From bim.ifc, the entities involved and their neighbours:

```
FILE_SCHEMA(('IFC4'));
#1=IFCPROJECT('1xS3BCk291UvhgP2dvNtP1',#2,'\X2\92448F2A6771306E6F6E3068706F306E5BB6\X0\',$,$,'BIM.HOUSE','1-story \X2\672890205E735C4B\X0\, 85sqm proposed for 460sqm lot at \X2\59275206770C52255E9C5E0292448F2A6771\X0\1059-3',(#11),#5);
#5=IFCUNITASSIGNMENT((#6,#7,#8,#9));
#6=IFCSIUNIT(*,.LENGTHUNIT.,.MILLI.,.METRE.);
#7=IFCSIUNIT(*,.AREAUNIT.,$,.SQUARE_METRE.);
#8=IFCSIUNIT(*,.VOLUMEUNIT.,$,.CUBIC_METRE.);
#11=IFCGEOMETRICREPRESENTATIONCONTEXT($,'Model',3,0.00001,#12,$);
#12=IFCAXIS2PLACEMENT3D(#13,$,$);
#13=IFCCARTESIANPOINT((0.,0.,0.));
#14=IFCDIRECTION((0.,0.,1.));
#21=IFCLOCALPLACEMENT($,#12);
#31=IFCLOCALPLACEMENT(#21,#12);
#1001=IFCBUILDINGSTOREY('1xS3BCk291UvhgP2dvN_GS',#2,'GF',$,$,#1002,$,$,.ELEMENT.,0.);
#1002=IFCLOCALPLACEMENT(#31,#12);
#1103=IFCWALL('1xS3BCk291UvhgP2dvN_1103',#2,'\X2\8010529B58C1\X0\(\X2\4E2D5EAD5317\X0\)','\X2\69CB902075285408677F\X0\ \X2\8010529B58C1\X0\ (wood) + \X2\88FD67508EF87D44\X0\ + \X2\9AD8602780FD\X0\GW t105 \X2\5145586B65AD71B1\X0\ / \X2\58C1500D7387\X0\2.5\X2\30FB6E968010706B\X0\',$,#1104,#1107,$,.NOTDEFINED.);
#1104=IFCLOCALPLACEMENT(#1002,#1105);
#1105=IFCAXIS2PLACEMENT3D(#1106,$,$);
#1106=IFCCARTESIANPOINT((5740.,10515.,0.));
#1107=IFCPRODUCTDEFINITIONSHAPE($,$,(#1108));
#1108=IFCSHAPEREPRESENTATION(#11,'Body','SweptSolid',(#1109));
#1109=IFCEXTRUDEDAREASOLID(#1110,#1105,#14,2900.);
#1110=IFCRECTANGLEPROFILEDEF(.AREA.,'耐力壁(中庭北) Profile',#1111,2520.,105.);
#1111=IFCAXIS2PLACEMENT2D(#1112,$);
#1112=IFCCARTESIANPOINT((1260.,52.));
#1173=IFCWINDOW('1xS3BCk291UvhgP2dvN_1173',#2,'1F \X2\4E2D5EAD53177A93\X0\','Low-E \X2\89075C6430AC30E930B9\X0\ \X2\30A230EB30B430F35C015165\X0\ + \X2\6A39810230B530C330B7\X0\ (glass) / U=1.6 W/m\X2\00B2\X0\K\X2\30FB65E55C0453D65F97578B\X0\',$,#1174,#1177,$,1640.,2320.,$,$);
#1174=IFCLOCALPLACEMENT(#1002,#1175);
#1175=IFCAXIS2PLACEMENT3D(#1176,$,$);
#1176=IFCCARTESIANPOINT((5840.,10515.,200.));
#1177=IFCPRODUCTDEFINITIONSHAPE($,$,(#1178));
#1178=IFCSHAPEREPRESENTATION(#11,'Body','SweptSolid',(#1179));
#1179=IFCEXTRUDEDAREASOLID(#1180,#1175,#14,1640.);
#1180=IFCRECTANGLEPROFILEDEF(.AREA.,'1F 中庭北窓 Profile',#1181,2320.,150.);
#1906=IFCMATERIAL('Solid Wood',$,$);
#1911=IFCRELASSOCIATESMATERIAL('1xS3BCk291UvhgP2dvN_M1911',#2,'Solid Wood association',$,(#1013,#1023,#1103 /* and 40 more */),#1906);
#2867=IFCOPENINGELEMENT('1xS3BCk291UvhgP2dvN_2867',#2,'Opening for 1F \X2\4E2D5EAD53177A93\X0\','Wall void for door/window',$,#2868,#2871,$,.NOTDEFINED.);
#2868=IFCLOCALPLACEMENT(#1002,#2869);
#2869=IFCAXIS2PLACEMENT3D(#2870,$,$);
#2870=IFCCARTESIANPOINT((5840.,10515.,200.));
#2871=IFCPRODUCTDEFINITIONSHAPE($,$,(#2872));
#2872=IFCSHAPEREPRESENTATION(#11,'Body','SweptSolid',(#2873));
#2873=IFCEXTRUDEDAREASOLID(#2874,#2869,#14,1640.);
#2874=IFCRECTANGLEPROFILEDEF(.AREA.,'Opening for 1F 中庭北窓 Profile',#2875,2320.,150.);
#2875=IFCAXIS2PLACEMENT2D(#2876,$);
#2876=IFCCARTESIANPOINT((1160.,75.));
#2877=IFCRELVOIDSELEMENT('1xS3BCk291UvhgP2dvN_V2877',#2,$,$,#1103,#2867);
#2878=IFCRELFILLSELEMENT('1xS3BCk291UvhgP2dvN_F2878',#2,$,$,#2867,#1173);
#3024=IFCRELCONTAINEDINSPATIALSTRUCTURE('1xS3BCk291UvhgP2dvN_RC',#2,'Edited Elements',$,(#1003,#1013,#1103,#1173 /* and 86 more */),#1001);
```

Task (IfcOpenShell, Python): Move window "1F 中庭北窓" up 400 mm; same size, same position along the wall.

```python
import numpy as np
import ifcopenshell
import ifcopenshell.api.geometry
import ifcopenshell.util.placement
import ifcopenshell.util.unit

model = ifcopenshell.open("bim.ifc")
unit_scale = ifcopenshell.util.unit.calculate_unit_scale(model)

window = model.by_guid("1xS3BCk291UvhgP2dvN_1173")
opening = window.FillsVoids[0].RelatingOpeningElement
dz = 400.0

shift = np.array([0.0, 0.0, dz])
# The window is not placed relative to its opening, so move both.
for product in (opening, window):
    matrix = ifcopenshell.util.placement.get_local_placement(product.ObjectPlacement)
    matrix[:3, 3] += shift
    ifcopenshell.api.geometry.edit_object_placement(model, product=product, matrix=matrix, is_si=False)

print(f"moved by {dz * unit_scale:+.3f} m")

model.write("bim_v2.ifc")
```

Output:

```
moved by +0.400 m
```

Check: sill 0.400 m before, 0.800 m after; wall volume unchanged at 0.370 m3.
